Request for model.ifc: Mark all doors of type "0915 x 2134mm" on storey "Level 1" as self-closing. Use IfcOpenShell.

First a look at what the model holds.

```python
import ifcopenshell
import ifcopenshell.util.element

model = ifcopenshell.open("model.ifc")
print(model.schema)
storey = next(s for s in model.by_type("IfcBuildingStorey") if s.Name == "Level 1")
doors = [e for e in ifcopenshell.util.element.get_decomposition(storey) if e.is_a("IfcDoor")]
seen = {}
for e in doors:
    element_type = ifcopenshell.util.element.get_type(e)
    key = (element_type.Name if element_type != e and element_type else None, ifcopenshell.util.element.get_pset(e, "Pset_DoorCommon", "SelfClosing"))
    seen[key] = seen.get(key, 0) + 1
for (name, value), count in sorted(seen.items(), key=str):
    print(count, "x", name, "|", value)
```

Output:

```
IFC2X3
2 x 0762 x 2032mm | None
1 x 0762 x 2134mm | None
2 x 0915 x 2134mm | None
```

```python
import ifcopenshell
import ifcopenshell.api.pset
import ifcopenshell.util.element

model = ifcopenshell.open("model.ifc")

storey = next(s for s in model.by_type("IfcBuildingStorey") if s.Name == "Level 1")
doors = [e for e in ifcopenshell.util.element.get_decomposition(storey) if e.is_a("IfcDoor")]

count = 0
for e in doors:
    element_type = ifcopenshell.util.element.get_type(e)
    if element_type in (None, e) or element_type.Name != "0915 x 2134mm":
        continue
    # add_pset returns the element's existing set when there is one.
    pset = ifcopenshell.api.pset.add_pset(model, product=e, name="Pset_DoorCommon")
    ifcopenshell.api.pset.edit_pset(model, pset=pset, properties={"SelfClosing": True})
    count += 1

print(count, "doors updated")

model.write("model_v2.ifc")
```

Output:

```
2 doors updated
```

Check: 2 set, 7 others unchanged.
